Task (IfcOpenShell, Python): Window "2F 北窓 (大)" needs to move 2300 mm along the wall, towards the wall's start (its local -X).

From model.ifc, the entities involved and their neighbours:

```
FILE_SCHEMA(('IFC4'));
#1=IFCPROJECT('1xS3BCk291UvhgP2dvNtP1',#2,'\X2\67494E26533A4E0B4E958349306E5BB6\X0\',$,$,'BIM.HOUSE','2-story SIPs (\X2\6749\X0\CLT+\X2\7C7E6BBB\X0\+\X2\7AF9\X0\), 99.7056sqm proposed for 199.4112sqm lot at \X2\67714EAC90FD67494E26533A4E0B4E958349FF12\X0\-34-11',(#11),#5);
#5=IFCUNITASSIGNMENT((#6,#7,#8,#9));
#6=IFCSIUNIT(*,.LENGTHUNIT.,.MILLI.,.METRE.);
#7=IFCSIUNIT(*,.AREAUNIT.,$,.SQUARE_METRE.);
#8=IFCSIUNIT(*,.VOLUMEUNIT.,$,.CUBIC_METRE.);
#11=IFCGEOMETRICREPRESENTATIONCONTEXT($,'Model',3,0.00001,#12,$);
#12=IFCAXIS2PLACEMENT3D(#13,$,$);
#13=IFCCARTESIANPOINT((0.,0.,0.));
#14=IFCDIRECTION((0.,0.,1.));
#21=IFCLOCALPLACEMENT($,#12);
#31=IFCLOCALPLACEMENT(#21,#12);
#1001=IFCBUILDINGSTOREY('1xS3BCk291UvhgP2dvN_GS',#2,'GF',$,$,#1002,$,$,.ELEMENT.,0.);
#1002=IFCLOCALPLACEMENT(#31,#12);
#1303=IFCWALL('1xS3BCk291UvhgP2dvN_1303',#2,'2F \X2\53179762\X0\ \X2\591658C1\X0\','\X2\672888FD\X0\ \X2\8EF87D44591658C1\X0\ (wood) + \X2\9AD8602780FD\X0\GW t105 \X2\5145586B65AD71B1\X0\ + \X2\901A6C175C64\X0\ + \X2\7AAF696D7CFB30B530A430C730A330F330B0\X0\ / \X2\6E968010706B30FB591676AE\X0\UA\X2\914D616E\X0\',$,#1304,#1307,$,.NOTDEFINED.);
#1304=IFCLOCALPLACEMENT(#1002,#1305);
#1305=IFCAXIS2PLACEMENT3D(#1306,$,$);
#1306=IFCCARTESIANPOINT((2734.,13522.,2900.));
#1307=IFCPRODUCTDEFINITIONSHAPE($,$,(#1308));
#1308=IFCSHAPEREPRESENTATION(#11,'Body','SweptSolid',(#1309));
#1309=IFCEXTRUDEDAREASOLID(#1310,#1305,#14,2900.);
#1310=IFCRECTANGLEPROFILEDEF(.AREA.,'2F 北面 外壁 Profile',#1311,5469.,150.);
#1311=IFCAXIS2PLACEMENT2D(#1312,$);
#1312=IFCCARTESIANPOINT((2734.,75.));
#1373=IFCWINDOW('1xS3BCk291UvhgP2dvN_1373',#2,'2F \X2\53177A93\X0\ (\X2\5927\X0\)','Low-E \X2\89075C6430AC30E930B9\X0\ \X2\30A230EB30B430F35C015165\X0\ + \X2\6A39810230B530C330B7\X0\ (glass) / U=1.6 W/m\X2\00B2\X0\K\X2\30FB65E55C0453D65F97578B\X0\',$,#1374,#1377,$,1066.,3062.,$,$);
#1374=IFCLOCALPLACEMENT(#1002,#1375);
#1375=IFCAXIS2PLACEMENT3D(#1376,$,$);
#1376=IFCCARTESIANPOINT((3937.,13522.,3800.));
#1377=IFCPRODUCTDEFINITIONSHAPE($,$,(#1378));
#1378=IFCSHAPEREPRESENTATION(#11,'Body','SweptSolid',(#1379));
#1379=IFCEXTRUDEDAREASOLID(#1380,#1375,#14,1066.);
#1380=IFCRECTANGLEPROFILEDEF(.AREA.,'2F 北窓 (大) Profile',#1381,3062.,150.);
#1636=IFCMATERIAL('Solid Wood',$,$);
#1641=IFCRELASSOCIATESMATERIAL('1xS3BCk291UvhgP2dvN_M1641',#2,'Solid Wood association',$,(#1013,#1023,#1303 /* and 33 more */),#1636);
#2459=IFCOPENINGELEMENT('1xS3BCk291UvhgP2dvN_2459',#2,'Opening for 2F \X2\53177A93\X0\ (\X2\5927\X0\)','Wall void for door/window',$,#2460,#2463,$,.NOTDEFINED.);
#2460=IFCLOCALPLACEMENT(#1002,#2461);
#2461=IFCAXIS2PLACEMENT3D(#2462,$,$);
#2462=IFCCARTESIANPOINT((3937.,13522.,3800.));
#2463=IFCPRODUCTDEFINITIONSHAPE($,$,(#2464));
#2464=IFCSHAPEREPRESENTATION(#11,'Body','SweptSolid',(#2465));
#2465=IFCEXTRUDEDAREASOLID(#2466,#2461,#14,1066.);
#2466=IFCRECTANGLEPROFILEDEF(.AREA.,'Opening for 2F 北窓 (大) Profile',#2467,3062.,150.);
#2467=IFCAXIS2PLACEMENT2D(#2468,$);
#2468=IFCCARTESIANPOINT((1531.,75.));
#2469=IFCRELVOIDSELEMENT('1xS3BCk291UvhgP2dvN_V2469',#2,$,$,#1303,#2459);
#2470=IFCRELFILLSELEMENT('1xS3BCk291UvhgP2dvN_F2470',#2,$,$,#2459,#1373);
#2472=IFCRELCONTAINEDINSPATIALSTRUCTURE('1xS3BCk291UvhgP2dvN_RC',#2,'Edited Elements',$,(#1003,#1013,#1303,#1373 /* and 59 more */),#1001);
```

```python
import ifcopenshell
import ifcopenshell.api.geometry
import ifcopenshell.util.placement

model = ifcopenshell.open("model.ifc")

window = model.by_id(1373)
opening = window.FillsVoids[0].RelatingOpeningElement
wall = opening.VoidsElements[0].RelatingBuildingElement

wall_matrix = ifcopenshell.util.placement.get_local_placement(wall.ObjectPlacement)
shift = wall_matrix[:3, 0] * -2300.0
before = ifcopenshell.util.placement.get_local_placement(window.ObjectPlacement)[:3, 3].copy()

# The window is not placed relative to its opening, so move both.
for product in (opening, window):
    matrix = ifcopenshell.util.placement.get_local_placement(product.ObjectPlacement)
    matrix[:3, 3] += shift
    ifcopenshell.api.geometry.edit_object_placement(model, product=product, matrix=matrix, is_si=False)

after = ifcopenshell.util.placement.get_local_placement(window.ObjectPlacement)[:3, 3]
print("window moved by", (after - before).round(3) + 0.0)

model.write("model_edited.ifc")
```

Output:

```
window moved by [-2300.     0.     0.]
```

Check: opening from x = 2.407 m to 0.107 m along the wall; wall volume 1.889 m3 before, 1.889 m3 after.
